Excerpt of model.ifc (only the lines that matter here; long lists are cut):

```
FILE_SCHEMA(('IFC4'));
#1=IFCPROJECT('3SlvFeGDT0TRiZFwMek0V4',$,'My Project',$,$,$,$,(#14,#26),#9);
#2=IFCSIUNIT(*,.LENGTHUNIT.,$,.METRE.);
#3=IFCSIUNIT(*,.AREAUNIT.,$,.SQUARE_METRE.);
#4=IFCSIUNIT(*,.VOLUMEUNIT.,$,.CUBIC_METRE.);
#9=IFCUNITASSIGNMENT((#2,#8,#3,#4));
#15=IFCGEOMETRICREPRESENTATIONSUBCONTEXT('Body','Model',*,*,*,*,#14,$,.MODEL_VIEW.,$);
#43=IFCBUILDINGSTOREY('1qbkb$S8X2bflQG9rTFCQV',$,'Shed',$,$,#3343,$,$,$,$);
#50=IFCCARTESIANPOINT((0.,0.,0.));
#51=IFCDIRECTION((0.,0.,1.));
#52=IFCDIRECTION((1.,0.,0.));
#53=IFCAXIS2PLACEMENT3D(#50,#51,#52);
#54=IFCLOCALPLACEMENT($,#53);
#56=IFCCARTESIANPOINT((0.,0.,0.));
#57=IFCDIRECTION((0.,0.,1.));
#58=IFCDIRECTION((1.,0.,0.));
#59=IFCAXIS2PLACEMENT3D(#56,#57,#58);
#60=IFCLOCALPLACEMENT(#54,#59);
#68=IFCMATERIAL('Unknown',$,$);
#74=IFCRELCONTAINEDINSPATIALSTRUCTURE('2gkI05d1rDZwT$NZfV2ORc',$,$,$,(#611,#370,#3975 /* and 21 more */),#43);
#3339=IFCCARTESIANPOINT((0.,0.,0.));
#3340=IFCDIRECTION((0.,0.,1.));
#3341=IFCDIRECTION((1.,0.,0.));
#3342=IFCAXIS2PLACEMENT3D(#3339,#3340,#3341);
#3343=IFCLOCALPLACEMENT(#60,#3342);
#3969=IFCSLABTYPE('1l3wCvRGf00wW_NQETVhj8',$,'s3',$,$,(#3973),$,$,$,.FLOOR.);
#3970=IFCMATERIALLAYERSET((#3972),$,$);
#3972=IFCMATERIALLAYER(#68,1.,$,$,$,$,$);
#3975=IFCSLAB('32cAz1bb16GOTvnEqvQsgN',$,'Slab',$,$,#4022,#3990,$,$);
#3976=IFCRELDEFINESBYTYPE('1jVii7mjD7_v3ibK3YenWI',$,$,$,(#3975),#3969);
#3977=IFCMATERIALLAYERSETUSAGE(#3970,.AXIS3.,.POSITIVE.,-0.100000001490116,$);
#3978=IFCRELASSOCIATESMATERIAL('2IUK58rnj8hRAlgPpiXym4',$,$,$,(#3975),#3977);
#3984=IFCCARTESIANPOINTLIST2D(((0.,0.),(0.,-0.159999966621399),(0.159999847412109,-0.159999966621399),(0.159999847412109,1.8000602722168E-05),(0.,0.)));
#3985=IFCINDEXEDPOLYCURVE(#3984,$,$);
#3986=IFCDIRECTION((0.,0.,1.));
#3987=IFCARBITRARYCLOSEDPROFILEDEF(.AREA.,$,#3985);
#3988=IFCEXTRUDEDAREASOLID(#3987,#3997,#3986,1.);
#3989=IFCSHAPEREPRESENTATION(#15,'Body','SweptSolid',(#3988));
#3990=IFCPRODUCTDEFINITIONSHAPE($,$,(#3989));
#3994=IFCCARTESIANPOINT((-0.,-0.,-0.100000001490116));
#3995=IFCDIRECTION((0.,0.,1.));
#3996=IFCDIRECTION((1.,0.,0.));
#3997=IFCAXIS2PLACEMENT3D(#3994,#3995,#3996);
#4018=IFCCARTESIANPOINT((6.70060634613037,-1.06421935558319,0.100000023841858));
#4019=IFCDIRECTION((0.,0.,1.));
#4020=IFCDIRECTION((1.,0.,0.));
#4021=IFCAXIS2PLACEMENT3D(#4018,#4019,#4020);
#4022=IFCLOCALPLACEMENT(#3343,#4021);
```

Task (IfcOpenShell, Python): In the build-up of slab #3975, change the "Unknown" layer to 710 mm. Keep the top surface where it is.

```python
import ifcopenshell
import ifcopenshell.util.element
import ifcopenshell.util.representation

model = ifcopenshell.open("model.ifc")

layer_set = model.by_id(3970)
layer = next(l for l in layer_set.MaterialLayers if l.Material and l.Material.Name == "Unknown")
change = 0.71 - layer.LayerThickness
layer.LayerThickness += change

# Geometry does not follow the layer set by itself.
slabs = [e for e in ifcopenshell.util.element.get_elements_by_material(model, layer_set) if e.is_a("IfcSlab")]
for slab in sorted(slabs, key=lambda e: e.id()):
    body = ifcopenshell.util.representation.get_representation(slab, "Model", "Body")
    solid = body.Items[0]
    old_depth = solid.Depth
    solid.Depth += change
    # Extruded upwards: lower the start of the extrusion so the top stays.
    x, y, z = solid.Position.Location.Coordinates
    solid.Position.Location = model.createIfcCartesianPoint((x, y, z - change))
    print(slab.id(), f"{old_depth:g} -> {solid.Depth:g}")

# The layers are counted up from the underside, which has moved.
for usage in {ifcopenshell.util.element.get_material(slab) for slab in slabs}:
    usage.OffsetFromReferenceLine -= change

model.write("model_edited.ifc")
```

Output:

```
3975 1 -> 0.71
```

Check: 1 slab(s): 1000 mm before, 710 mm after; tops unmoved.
